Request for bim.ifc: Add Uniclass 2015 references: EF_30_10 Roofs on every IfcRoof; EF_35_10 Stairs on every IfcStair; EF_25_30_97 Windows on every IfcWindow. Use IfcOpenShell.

First a look at what the model holds.

```python
import ifcopenshell

model = ifcopenshell.open("bim.ifc")
print(model.schema)
print("classifications:", [c.Name for c in model.by_type("IfcClassification")])
for ifc_class in ("IfcDoor", "IfcRoof", "IfcStair", "IfcWall", "IfcWindow"):
    print(ifc_class, len(model.by_type(ifc_class)))
```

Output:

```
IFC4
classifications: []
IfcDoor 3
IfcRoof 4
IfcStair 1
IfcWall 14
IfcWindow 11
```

```python
import ifcopenshell
import ifcopenshell.api.classification

model = ifcopenshell.open("bim.ifc")

system = ifcopenshell.api.classification.add_classification(model, classification="Uniclass 2015")

codes = {
    "IfcRoof": ("EF_30_10", "Roofs"),
    "IfcStair": ("EF_35_10", "Stairs"),
    "IfcWindow": ("EF_25_30_97", "Windows"),
}
for ifc_class, (code, name) in codes.items():
    products = model.by_type(ifc_class)
    ifcopenshell.api.classification.add_reference(
        model, products=products, classification=system, identification=code, name=name
    )
    print(code, len(products))

model.write("bim-out.ifc")
```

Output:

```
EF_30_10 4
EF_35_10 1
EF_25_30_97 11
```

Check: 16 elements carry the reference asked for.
